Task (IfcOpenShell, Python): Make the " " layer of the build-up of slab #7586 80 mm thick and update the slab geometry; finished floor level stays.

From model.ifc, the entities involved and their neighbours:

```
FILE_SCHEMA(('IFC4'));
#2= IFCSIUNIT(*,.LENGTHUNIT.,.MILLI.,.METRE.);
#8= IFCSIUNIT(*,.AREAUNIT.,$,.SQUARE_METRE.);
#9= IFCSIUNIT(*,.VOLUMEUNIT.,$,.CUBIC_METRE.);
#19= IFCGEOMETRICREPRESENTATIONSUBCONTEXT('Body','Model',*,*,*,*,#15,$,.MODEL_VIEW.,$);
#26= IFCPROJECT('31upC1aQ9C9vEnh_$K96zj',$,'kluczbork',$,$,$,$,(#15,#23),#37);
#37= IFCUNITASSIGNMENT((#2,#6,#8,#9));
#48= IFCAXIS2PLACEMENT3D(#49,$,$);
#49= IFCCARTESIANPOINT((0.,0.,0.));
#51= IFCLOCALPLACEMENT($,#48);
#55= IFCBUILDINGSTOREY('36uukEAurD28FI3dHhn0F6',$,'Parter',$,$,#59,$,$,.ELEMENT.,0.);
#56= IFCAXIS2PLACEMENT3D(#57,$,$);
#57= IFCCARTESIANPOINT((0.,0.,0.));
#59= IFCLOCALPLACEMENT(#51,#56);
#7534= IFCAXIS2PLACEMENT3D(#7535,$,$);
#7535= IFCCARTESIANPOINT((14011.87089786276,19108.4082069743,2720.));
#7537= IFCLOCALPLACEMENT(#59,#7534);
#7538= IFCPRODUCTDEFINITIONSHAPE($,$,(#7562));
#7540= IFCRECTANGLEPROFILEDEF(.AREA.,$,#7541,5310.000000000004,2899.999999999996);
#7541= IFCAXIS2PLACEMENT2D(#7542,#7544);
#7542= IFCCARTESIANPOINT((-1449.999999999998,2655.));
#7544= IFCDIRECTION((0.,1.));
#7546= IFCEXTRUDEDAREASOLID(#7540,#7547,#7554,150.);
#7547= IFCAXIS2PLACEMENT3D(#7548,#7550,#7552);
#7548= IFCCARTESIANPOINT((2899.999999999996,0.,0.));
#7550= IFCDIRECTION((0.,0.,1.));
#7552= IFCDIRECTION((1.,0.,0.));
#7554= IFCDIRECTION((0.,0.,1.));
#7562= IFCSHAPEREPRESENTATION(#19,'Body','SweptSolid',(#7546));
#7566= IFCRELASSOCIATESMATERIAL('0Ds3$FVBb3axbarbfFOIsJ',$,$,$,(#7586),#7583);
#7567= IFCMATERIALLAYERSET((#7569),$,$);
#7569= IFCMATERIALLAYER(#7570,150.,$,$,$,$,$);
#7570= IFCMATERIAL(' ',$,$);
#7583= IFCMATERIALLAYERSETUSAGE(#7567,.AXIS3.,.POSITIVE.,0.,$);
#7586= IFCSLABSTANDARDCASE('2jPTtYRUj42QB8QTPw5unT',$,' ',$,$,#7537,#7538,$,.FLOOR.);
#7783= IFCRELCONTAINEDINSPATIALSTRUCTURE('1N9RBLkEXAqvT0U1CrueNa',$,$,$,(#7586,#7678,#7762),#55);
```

```python
import ifcopenshell
import ifcopenshell.util.element
import ifcopenshell.util.representation
import ifcopenshell.util.unit

model = ifcopenshell.open("model.ifc")
unit_scale = ifcopenshell.util.unit.calculate_unit_scale(model)

layer_set = model.by_id(7567)
layer = next(l for l in layer_set.MaterialLayers if l.Material and l.Material.Name == " ")
change = 0.08 / unit_scale - layer.LayerThickness
layer.LayerThickness += change

# Geometry does not follow the layer set by itself.
slabs = [e for e in ifcopenshell.util.element.get_elements_by_material(model, layer_set) if e.is_a("IfcSlab")]
for slab in sorted(slabs, key=lambda e: e.id()):
    body = ifcopenshell.util.representation.get_representation(slab, "Model", "Body")
    solid = body.Items[0]
    old_depth = solid.Depth
    solid.Depth += change
    # Extruded upwards: lower the start of the extrusion so the top stays.
    x, y, z = solid.Position.Location.Coordinates
    solid.Position.Location = model.createIfcCartesianPoint((x, y, z - change))
    print(slab.id(), f"{old_depth:g} -> {solid.Depth:g}")

# The layers are counted up from the underside, which has moved.
for usage in {ifcopenshell.util.element.get_material(slab) for slab in slabs}:
    usage.OffsetFromReferenceLine -= change

model.write("model_rev.ifc")
```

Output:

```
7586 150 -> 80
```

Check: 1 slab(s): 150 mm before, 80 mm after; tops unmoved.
